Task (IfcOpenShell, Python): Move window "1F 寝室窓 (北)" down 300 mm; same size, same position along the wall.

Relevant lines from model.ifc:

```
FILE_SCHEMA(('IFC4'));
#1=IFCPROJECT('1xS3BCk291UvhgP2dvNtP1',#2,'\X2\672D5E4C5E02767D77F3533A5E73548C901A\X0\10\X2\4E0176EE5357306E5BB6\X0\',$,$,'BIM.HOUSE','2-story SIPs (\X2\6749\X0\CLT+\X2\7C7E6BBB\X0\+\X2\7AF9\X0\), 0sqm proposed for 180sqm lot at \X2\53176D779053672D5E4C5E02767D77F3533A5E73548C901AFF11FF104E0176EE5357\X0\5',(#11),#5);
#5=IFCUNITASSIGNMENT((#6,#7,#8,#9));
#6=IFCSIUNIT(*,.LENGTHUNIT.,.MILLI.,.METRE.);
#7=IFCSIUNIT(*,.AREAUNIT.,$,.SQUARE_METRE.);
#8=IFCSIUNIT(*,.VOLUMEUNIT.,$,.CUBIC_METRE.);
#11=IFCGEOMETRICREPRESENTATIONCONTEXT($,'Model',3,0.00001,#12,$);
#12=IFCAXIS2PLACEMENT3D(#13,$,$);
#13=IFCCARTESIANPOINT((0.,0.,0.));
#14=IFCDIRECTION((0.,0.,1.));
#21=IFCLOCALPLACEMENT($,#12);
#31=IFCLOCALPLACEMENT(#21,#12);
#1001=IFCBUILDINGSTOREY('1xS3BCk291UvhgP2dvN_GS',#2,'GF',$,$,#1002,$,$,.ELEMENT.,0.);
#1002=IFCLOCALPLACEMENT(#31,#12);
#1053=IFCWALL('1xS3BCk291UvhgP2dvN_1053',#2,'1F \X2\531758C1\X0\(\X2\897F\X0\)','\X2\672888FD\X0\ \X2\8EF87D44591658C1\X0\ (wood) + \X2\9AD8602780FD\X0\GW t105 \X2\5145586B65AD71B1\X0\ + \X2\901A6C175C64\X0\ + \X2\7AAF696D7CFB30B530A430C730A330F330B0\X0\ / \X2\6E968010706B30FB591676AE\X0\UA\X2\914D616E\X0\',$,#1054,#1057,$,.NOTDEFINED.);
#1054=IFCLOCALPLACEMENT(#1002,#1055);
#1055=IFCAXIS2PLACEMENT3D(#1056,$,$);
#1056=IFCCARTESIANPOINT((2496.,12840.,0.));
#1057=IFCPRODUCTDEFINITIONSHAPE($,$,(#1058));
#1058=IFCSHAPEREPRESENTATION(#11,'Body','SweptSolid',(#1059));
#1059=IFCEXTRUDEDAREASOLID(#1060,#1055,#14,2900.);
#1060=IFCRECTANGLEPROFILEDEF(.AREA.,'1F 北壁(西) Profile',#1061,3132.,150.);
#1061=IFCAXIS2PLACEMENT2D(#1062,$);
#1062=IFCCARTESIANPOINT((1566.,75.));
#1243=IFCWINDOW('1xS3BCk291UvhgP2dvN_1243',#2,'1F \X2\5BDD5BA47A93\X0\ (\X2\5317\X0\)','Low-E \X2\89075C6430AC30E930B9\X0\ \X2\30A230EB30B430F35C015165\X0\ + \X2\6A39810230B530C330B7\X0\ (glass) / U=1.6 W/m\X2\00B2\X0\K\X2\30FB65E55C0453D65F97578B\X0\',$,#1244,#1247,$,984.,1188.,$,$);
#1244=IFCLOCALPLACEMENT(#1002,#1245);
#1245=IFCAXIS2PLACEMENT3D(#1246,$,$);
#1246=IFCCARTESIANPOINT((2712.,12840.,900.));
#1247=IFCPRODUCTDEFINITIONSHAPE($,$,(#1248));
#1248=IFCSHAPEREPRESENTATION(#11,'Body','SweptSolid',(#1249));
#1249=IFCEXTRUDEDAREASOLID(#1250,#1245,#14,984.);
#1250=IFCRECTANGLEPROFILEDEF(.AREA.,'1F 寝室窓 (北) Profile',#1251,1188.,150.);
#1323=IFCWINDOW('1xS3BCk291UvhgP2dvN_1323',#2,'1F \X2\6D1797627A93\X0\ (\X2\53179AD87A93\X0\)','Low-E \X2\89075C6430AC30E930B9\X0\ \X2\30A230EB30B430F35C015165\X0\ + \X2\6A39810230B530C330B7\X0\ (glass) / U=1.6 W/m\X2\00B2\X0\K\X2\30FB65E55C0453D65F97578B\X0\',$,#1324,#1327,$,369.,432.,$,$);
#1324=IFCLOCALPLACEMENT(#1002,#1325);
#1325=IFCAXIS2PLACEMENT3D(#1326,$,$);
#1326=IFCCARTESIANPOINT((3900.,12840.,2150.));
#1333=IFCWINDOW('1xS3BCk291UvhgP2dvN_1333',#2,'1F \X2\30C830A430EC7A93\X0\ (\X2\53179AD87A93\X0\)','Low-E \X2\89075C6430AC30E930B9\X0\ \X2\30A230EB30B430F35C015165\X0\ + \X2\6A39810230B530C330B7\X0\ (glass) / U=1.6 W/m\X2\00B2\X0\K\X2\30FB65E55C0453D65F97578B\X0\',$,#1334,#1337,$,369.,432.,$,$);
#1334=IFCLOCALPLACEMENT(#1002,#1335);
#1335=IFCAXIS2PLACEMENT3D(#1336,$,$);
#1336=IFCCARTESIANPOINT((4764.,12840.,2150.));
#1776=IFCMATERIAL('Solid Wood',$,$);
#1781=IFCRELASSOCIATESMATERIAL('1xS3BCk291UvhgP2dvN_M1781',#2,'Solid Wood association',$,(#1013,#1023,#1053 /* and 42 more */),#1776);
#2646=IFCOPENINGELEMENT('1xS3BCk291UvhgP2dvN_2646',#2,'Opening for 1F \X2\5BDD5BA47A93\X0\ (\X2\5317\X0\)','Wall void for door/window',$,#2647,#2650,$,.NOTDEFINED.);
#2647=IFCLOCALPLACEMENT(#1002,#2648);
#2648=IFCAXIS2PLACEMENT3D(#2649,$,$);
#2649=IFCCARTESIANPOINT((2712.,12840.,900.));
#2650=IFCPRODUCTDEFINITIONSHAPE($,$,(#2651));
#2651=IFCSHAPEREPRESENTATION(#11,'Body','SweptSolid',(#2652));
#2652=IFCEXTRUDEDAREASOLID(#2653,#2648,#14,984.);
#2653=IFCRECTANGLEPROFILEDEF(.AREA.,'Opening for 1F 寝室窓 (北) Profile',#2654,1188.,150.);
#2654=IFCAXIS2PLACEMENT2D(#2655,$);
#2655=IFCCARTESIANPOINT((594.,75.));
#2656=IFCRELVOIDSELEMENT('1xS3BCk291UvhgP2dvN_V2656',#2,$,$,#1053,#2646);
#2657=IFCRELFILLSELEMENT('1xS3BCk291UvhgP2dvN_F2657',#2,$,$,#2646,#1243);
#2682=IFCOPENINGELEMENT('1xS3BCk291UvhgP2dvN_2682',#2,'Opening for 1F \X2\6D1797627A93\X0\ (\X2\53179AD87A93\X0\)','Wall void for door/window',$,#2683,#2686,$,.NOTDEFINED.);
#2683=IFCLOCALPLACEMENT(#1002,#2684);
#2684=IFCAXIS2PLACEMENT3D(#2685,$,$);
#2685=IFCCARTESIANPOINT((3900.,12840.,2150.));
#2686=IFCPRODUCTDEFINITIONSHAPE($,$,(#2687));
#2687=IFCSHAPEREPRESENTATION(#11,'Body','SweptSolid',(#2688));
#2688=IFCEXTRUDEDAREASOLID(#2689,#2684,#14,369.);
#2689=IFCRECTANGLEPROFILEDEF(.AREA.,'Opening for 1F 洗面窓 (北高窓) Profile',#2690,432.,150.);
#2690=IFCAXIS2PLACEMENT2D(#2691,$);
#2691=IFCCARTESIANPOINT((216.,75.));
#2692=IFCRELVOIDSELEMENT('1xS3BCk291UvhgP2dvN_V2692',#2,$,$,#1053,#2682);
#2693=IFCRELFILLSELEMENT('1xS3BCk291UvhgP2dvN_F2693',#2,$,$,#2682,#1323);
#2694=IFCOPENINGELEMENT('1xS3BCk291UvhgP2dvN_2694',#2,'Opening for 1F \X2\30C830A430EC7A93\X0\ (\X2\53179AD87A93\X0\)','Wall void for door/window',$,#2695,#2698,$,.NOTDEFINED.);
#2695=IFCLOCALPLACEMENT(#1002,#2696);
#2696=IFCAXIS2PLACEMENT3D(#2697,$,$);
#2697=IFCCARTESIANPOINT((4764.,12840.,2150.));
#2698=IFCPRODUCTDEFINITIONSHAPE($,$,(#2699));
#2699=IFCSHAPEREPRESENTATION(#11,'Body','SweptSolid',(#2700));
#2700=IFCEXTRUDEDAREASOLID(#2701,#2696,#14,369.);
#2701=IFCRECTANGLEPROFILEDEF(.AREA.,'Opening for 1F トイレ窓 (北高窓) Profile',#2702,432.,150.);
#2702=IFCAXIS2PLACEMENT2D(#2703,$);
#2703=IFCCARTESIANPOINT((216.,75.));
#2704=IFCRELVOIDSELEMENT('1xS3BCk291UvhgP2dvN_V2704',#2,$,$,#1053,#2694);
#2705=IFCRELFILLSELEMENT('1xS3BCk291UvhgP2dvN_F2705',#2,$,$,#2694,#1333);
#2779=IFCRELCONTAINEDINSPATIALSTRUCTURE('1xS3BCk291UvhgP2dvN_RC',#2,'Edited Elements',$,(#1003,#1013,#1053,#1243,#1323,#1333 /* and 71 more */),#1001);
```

```python
import numpy as np
import ifcopenshell
import ifcopenshell.api.geometry
import ifcopenshell.util.placement
import ifcopenshell.util.unit

model = ifcopenshell.open("model.ifc")
unit_scale = ifcopenshell.util.unit.calculate_unit_scale(model)

window = model.by_guid("1xS3BCk291UvhgP2dvN_1243")
opening = window.FillsVoids[0].RelatingOpeningElement
dz = -300.0

shift = np.array([0.0, 0.0, dz])
# The window is not placed relative to its opening, so move both.
for product in (opening, window):
    matrix = ifcopenshell.util.placement.get_local_placement(product.ObjectPlacement)
    matrix[:3, 3] += shift
    ifcopenshell.api.geometry.edit_object_placement(model, product=product, matrix=matrix, is_si=False)

print(f"moved by {dz * unit_scale:+.3f} m")

model.write("model-out.ifc")
```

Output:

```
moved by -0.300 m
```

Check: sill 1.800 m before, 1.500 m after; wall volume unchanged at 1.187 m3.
